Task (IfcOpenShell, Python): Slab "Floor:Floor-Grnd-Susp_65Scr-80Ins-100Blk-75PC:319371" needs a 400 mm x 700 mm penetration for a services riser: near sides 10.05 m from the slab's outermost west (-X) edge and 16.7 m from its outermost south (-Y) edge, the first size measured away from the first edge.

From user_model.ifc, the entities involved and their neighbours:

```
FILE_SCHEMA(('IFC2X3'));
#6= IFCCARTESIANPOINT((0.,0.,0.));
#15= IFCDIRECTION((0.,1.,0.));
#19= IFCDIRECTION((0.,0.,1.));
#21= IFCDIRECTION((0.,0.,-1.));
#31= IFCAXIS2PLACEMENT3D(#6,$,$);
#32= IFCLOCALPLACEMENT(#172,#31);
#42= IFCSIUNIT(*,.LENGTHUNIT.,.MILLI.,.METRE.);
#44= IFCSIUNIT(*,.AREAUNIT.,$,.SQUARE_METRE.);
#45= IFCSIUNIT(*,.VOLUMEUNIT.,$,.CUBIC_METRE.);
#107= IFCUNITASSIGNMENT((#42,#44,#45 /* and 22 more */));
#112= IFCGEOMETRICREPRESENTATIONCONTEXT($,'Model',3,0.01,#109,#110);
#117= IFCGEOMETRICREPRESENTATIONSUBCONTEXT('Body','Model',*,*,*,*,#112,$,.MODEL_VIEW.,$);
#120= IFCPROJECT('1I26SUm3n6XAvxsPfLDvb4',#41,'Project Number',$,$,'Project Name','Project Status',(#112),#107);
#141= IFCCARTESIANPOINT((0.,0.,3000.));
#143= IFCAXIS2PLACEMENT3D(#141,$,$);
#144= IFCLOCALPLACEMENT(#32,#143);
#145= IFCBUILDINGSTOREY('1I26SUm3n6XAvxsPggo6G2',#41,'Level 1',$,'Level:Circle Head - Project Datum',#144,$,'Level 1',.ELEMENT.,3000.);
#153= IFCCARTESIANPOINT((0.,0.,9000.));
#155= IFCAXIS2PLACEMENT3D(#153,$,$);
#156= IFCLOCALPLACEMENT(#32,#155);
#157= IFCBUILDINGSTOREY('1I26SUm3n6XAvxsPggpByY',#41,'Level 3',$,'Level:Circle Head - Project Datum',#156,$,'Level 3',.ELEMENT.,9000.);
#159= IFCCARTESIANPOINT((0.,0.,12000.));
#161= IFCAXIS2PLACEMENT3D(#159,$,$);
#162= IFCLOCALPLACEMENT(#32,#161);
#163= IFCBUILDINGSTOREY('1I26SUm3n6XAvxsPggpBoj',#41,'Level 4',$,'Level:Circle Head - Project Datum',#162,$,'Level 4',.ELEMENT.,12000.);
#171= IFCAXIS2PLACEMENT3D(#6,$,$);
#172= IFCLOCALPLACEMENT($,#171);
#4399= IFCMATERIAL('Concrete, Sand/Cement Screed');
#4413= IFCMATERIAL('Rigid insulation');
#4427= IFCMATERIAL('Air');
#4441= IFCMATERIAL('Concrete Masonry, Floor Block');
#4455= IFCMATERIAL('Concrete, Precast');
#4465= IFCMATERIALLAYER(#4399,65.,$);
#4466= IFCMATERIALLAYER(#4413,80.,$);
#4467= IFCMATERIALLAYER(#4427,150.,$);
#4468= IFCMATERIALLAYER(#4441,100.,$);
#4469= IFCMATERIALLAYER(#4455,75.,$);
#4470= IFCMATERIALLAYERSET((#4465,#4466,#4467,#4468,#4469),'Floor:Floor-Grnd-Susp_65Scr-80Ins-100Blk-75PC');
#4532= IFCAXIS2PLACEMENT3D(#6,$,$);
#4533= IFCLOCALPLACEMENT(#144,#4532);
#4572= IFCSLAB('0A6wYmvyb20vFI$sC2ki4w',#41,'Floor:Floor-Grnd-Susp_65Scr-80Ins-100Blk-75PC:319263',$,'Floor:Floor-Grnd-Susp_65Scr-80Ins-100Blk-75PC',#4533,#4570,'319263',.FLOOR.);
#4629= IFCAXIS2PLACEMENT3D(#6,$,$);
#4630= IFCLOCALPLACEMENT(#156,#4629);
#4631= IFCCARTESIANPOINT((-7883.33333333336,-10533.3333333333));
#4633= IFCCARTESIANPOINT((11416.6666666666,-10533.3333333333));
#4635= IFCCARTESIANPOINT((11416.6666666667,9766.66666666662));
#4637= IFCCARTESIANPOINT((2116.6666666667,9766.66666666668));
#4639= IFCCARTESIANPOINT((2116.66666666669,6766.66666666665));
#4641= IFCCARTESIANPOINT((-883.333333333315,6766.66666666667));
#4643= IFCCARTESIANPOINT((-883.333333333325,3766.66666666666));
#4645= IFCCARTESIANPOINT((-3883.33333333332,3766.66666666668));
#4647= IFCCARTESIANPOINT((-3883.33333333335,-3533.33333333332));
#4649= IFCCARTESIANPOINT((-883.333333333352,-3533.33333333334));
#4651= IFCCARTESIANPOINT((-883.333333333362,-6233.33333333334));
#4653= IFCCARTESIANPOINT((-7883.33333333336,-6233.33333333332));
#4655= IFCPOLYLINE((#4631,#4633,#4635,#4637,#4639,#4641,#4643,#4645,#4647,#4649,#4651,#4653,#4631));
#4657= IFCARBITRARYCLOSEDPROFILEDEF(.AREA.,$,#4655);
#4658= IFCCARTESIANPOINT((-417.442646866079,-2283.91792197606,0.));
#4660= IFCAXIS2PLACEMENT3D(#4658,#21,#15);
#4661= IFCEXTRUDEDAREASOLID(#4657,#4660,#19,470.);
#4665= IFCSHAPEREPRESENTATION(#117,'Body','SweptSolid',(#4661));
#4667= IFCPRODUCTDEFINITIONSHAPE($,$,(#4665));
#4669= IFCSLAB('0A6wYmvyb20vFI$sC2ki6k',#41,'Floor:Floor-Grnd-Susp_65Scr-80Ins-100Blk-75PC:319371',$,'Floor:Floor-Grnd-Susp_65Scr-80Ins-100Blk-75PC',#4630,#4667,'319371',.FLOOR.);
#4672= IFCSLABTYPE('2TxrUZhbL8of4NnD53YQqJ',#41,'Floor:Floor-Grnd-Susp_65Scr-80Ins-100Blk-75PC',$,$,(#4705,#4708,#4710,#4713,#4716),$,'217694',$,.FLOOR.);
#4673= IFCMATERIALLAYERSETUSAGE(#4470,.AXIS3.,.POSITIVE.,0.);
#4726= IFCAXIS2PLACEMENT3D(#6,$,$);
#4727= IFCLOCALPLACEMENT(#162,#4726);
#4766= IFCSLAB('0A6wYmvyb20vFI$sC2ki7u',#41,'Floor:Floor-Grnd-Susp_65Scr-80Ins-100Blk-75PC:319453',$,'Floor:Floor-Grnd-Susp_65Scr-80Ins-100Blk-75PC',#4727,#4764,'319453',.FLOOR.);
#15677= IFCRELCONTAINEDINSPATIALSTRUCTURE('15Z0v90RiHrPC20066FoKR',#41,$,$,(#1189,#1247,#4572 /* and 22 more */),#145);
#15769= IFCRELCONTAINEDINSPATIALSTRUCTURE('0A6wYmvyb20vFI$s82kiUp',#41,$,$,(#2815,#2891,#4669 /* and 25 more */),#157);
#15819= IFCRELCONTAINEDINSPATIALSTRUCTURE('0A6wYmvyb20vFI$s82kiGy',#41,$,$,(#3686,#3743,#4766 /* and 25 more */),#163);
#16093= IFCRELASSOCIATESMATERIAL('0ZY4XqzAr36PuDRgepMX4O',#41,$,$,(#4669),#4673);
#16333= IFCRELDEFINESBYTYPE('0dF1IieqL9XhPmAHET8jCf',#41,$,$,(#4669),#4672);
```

```python
import numpy as np
import ifcopenshell
import ifcopenshell.api.feature
import ifcopenshell.api.geometry
import ifcopenshell.api.root
import ifcopenshell.geom
import ifcopenshell.util.placement
import ifcopenshell.util.representation
import ifcopenshell.util.shape
import ifcopenshell.util.unit

model = ifcopenshell.open("user_model.ifc")
unit_scale = ifcopenshell.util.unit.calculate_unit_scale(model)
settings = ifcopenshell.geom.settings()


def volume(element):
    """Net volume in cubic metres, openings subtracted."""
    shape = ifcopenshell.geom.create_shape(settings, element)
    return ifcopenshell.util.shape.get_volume(shape.geometry)


slab = model.by_id(4669)
before = volume(slab)

# Extent in the slab's own axes, in metres. The edges named are its -X and -Y sides.
slab_shape = ifcopenshell.geom.create_shape(settings, slab)
vertices = ifcopenshell.util.shape.get_vertices(slab_shape.geometry)
x_min, y_min, bottom = vertices.min(axis=0)
top = vertices[:, 2].max()

opening = ifcopenshell.api.root.create_entity(model, ifc_class="IfcOpeningElement", name="Services riser opening")
context = ifcopenshell.util.representation.get_context(model, "Model", "Body", "MODEL_VIEW")
width, depth = 0.4, 0.7
outline = [(0.0, 0.0), (width, 0.0), (width, depth), (0.0, depth), (0.0, 0.0)]
# Overshoot both faces by 50 mm so the cut is clean.
shape = ifcopenshell.api.geometry.add_slab_representation(
    model, context=context, depth=top - bottom + 0.1, polyline=outline
)
ifcopenshell.api.geometry.assign_representation(model, product=opening, representation=shape)

matrix = ifcopenshell.util.placement.get_local_placement(slab.ObjectPlacement)
matrix[:, 3] = matrix @ np.append(np.array([x_min + 10.05, y_min + 16.7, bottom - 0.05]) / unit_scale, 1.0)
ifcopenshell.api.geometry.edit_object_placement(model, product=opening, matrix=matrix, is_si=False)
ifcopenshell.api.feature.add_feature(model, feature=opening, element=slab)

after = volume(slab)

print(f"slab volume {before:.3f} -> {after:.3f} m3")

model.write("user_model_updated.ifc")
```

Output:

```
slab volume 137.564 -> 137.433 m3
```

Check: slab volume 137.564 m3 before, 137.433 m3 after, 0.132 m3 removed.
